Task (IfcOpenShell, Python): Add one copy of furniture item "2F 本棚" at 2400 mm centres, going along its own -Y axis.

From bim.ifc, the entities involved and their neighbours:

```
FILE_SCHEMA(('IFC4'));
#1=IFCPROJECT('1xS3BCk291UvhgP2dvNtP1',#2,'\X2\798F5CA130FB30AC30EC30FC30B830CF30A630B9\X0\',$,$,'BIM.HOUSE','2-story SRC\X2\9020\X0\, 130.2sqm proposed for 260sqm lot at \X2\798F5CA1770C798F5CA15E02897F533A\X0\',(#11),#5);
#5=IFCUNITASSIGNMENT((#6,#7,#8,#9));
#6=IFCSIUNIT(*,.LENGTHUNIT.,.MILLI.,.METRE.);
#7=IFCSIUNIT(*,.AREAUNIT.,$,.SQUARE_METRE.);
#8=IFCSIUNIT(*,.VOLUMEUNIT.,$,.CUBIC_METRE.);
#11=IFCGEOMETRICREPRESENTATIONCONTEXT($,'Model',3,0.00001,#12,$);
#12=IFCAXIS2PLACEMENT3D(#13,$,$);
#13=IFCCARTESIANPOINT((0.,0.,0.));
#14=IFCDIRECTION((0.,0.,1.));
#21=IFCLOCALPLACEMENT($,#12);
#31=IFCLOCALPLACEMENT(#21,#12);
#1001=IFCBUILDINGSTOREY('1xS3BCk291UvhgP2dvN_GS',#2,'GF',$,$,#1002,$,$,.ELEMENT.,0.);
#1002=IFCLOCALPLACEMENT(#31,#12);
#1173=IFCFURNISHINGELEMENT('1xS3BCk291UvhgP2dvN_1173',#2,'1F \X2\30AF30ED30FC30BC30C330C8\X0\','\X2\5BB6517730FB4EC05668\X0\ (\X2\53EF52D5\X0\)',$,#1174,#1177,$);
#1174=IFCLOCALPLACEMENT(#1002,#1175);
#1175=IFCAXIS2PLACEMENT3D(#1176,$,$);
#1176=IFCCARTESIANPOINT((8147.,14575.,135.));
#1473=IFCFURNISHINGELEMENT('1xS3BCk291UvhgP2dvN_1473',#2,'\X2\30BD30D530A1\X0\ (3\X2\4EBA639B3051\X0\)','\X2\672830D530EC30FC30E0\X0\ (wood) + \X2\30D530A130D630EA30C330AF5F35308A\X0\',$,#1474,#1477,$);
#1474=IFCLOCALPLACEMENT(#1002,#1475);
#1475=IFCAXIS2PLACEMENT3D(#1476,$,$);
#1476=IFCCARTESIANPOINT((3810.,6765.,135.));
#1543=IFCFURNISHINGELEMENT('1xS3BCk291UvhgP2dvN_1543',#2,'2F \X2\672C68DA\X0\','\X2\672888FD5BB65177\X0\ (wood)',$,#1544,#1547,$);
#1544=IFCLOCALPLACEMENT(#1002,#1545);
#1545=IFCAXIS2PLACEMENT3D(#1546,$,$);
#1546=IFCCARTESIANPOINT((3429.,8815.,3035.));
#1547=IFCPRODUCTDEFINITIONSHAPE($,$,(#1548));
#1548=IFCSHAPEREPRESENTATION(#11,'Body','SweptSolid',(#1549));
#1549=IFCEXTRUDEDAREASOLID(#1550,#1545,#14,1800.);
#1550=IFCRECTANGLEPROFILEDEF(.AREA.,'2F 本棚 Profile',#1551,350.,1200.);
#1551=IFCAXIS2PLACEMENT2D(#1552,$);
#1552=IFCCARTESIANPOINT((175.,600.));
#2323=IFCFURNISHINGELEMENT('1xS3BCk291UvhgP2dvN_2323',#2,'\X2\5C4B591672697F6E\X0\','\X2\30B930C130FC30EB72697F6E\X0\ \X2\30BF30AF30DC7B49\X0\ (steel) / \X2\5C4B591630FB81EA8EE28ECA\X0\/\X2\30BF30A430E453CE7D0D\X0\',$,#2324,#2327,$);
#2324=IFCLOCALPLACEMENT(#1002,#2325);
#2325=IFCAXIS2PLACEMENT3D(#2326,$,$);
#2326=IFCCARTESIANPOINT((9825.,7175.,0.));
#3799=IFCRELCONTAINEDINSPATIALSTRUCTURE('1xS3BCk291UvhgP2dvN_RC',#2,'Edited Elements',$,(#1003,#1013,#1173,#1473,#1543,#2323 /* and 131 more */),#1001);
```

```python
import ifcopenshell
import ifcopenshell.api.geometry
import ifcopenshell.api.root
import ifcopenshell.util.element
import ifcopenshell.util.placement
import ifcopenshell.util.unit

model = ifcopenshell.open("bim.ifc")
unit_scale = ifcopenshell.util.unit.calculate_unit_scale(model)


def reuse_history(source, copy):
    """copy_class also copies each property set's owner history, people and application; keep the originals."""
    for rel in copy.IsDefinedBy:
        if rel.is_a("IfcRelDefinesByProperties") and (history := rel.RelatingPropertyDefinition.OwnerHistory):
            rel.RelatingPropertyDefinition.OwnerHistory = source.OwnerHistory
            ifcopenshell.util.element.remove_deep2(model, history)


source = model.by_id(1543)
base = ifcopenshell.util.placement.get_local_placement(source.ObjectPlacement)
step = -base[:3, 1] * 2.4 / unit_scale

for i in range(1, 2):
    copy = ifcopenshell.api.root.copy_class(model, product=source)
    copy.Representation = ifcopenshell.util.element.copy_deep(
        model, source.Representation, exclude=["IfcGeometricRepresentationContext", "IfcRepresentationMap"]
    )
    reuse_history(source, copy)
    matrix = base.copy()
    matrix[:3, 3] += i * step
    print("added at", matrix[:3, 3].round(3) + 0.0)
    ifcopenshell.api.geometry.edit_object_placement(model, product=copy, matrix=matrix, is_si=False)

model.write("bim_rev.ifc")
```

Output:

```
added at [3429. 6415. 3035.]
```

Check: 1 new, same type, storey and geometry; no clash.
